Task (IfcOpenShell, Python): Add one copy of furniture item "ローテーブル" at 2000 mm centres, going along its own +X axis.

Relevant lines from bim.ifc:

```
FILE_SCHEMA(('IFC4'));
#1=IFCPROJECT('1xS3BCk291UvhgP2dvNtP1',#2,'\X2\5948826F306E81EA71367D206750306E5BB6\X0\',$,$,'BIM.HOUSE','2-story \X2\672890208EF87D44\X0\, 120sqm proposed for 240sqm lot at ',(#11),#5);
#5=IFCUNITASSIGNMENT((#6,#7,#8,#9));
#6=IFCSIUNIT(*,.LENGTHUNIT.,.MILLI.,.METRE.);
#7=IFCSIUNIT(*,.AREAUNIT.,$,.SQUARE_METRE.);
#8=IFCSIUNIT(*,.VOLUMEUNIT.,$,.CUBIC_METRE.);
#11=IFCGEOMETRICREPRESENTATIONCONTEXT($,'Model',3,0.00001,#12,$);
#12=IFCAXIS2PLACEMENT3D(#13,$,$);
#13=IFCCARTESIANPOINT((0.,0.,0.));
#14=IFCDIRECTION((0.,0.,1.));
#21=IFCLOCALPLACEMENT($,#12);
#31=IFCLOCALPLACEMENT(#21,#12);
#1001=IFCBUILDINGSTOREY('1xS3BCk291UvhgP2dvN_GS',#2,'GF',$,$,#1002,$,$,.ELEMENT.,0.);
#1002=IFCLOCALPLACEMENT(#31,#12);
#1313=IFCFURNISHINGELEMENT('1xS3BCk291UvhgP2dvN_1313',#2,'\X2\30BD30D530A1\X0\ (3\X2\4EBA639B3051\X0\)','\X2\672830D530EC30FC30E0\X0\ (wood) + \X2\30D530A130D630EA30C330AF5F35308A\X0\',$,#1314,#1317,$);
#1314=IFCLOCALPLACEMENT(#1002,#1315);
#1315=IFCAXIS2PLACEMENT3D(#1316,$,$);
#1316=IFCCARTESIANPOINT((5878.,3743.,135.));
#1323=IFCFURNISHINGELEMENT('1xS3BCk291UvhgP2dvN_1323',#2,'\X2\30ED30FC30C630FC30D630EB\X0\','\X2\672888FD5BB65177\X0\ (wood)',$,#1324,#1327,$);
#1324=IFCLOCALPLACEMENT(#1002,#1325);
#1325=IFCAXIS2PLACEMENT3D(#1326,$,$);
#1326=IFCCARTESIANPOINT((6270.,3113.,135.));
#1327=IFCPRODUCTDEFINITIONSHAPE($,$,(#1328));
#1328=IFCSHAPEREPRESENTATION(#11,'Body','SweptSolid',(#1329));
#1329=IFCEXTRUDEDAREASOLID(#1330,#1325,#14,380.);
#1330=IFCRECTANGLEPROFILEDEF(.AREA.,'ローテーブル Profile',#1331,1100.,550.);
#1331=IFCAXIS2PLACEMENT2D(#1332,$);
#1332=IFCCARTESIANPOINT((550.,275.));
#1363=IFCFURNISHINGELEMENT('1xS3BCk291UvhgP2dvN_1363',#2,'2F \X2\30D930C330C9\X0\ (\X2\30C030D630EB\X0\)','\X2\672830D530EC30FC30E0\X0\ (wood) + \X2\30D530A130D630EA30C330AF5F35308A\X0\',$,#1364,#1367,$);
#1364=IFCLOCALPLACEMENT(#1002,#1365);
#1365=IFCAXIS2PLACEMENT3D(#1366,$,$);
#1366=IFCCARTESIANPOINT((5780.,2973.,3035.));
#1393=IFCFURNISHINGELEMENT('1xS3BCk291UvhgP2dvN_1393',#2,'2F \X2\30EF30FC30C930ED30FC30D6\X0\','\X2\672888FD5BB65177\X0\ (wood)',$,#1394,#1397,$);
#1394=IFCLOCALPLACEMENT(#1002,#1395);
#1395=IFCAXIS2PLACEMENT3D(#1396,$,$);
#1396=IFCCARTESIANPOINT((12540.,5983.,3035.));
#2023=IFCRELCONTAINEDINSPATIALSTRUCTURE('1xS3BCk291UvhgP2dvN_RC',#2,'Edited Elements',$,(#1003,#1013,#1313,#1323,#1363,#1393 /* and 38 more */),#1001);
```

```python
import ifcopenshell
import ifcopenshell.api.geometry
import ifcopenshell.api.root
import ifcopenshell.util.element
import ifcopenshell.util.placement
import ifcopenshell.util.unit

model = ifcopenshell.open("bim.ifc")
unit_scale = ifcopenshell.util.unit.calculate_unit_scale(model)


def reuse_history(source, copy):
    """copy_class also copies each property set's owner history, people and application; keep the originals."""
    for rel in copy.IsDefinedBy:
        if rel.is_a("IfcRelDefinesByProperties") and (history := rel.RelatingPropertyDefinition.OwnerHistory):
            rel.RelatingPropertyDefinition.OwnerHistory = source.OwnerHistory
            ifcopenshell.util.element.remove_deep2(model, history)


source = model.by_id(1323)
base = ifcopenshell.util.placement.get_local_placement(source.ObjectPlacement)
step = base[:3, 0] * 2 / unit_scale

for i in range(1, 2):
    copy = ifcopenshell.api.root.copy_class(model, product=source)
    copy.Representation = ifcopenshell.util.element.copy_deep(
        model, source.Representation, exclude=["IfcGeometricRepresentationContext", "IfcRepresentationMap"]
    )
    reuse_history(source, copy)
    matrix = base.copy()
    matrix[:3, 3] += i * step
    print("added at", matrix[:3, 3].round(3) + 0.0)
    ifcopenshell.api.geometry.edit_object_placement(model, product=copy, matrix=matrix, is_si=False)

model.write("bim_updated.ifc")
```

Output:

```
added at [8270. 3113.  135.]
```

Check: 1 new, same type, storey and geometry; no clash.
